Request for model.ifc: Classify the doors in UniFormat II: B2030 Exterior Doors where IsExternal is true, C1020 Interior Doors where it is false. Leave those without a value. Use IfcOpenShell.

First a look at what the model holds.

```python
import ifcopenshell
import ifcopenshell.util.element

model = ifcopenshell.open("model.ifc")
print(model.schema)
print("classifications:", [c.Name for c in model.by_type("IfcClassification")])
values = [ifcopenshell.util.element.get_pset(e, "Pset_DoorCommon", "IsExternal") for e in model.by_type("IfcDoor")]
for value in (True, False, None):
    print("IsExternal", value, values.count(value))
```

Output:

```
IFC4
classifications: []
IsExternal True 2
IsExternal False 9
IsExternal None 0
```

```python
import ifcopenshell
import ifcopenshell.api.classification
import ifcopenshell.util.element

model = ifcopenshell.open("model.ifc")

system = ifcopenshell.api.classification.add_classification(model, classification="UniFormat II")

doors = model.by_type("IfcDoor")
external = {e: ifcopenshell.util.element.get_pset(e, "Pset_DoorCommon", "IsExternal") for e in doors}
for flag, code, name in ((True, "B2030", "Exterior Doors"), (False, "C1020", "Interior Doors")):
    products = [e for e in doors if external[e] is flag]
    ifcopenshell.api.classification.add_reference(
        model, products=products, classification=system, identification=code, name=name
    )
    print(code, len(products))

model.write("model-out.ifc")
```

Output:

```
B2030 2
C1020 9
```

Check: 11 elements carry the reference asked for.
